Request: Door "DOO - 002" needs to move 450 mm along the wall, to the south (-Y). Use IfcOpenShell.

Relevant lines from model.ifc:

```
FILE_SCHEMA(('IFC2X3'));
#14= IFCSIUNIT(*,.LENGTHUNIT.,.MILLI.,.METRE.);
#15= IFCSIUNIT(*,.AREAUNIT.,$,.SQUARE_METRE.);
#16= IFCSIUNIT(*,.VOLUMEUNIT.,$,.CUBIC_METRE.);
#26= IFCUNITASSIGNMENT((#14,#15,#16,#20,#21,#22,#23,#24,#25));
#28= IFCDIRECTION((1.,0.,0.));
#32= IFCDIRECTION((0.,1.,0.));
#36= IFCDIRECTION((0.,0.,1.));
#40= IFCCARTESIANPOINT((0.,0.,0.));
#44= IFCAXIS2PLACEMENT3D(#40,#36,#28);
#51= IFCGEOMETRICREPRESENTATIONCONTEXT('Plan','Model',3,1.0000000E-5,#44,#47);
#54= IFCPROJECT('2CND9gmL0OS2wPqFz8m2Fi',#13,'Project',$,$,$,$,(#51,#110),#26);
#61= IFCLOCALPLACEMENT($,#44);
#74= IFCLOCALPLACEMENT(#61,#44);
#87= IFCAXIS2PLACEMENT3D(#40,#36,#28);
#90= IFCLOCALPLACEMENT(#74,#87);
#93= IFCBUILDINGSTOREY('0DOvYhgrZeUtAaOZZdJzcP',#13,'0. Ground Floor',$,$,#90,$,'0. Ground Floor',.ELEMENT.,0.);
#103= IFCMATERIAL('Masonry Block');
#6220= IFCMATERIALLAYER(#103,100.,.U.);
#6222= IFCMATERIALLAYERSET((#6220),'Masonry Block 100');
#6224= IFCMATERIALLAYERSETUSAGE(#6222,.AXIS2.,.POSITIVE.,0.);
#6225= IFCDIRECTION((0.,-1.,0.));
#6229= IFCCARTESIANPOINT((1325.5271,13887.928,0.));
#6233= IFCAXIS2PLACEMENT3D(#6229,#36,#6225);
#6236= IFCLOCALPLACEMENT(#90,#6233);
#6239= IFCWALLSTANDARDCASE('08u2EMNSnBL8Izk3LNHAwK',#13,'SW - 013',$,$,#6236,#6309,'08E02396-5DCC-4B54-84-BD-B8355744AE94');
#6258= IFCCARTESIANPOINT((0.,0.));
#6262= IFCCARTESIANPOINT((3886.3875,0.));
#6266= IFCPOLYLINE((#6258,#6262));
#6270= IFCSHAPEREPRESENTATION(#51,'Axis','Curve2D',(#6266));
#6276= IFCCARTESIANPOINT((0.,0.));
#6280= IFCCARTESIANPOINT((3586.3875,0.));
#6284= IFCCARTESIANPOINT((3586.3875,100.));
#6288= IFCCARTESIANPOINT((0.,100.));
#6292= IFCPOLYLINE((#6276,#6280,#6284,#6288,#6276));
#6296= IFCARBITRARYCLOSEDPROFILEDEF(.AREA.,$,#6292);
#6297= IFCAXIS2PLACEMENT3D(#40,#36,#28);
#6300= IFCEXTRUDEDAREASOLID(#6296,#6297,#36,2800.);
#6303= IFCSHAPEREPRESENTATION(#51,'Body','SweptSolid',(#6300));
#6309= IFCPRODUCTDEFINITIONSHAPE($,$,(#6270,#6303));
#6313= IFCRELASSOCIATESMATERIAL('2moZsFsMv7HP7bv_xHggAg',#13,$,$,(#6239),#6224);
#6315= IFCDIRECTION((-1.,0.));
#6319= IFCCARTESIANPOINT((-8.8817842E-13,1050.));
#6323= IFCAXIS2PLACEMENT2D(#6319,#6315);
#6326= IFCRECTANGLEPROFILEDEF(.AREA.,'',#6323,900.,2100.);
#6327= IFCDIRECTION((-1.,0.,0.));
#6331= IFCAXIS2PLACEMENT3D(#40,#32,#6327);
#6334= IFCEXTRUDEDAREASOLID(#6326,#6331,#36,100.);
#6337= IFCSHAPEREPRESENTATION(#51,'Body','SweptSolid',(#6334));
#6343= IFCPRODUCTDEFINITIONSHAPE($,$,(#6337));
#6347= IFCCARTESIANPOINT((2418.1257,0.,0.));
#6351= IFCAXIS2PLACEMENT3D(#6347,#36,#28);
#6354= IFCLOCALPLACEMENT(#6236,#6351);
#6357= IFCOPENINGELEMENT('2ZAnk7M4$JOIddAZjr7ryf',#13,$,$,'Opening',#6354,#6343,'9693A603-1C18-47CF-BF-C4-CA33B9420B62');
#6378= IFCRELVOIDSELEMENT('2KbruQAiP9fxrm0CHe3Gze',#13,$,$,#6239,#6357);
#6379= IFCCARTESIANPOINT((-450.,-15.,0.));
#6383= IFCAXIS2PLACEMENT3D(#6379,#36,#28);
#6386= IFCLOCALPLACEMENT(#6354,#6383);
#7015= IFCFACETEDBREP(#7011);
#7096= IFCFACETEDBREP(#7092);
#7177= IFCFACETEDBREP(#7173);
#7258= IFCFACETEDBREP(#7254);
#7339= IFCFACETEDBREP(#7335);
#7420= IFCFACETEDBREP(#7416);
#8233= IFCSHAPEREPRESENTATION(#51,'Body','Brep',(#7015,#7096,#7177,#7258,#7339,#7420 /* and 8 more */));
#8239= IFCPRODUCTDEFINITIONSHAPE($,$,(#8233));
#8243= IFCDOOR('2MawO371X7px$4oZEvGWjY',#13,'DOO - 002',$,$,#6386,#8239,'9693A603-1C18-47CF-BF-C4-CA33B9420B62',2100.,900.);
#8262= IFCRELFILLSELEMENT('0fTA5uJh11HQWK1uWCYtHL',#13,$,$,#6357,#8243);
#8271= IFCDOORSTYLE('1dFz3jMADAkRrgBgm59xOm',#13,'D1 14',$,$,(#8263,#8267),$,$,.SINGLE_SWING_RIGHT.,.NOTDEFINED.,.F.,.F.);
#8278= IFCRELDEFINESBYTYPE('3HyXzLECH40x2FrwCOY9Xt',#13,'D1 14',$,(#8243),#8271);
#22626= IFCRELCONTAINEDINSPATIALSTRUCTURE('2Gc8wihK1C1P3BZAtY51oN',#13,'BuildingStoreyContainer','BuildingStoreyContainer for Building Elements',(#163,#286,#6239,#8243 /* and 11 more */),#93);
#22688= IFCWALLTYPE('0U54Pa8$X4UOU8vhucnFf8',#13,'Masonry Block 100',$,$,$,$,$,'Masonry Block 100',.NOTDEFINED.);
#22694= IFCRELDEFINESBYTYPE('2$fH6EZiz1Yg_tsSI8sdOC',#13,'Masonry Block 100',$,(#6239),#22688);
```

```python
import ifcopenshell
import ifcopenshell.api.geometry
import ifcopenshell.util.placement
import ifcopenshell.util.unit

model = ifcopenshell.open("model.ifc")
unit_scale = ifcopenshell.util.unit.calculate_unit_scale(model)

door = model.by_guid("2MawO371X7px$4oZEvGWjY")
opening = door.FillsVoids[0].RelatingOpeningElement
wall = opening.VoidsElements[0].RelatingBuildingElement

wall_matrix = ifcopenshell.util.placement.get_local_placement(wall.ObjectPlacement)
shift = wall_matrix[:3, 0] * 0.45 / unit_scale
before = ifcopenshell.util.placement.get_local_placement(door.ObjectPlacement)[:3, 3].copy()

# The door is placed relative to its opening, so it follows when the opening moves.
matrix = ifcopenshell.util.placement.get_local_placement(opening.ObjectPlacement)
matrix[:3, 3] += shift
ifcopenshell.api.geometry.edit_object_placement(
    model, product=opening, matrix=matrix, is_si=False, should_transform_children=True
)

after = ifcopenshell.util.placement.get_local_placement(door.ObjectPlacement)[:3, 3]
print("door moved by", (after - before).round(3) + 0.0)

model.write("model_v2.ifc")
```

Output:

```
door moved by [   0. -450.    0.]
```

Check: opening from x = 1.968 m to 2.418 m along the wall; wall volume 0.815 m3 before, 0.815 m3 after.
